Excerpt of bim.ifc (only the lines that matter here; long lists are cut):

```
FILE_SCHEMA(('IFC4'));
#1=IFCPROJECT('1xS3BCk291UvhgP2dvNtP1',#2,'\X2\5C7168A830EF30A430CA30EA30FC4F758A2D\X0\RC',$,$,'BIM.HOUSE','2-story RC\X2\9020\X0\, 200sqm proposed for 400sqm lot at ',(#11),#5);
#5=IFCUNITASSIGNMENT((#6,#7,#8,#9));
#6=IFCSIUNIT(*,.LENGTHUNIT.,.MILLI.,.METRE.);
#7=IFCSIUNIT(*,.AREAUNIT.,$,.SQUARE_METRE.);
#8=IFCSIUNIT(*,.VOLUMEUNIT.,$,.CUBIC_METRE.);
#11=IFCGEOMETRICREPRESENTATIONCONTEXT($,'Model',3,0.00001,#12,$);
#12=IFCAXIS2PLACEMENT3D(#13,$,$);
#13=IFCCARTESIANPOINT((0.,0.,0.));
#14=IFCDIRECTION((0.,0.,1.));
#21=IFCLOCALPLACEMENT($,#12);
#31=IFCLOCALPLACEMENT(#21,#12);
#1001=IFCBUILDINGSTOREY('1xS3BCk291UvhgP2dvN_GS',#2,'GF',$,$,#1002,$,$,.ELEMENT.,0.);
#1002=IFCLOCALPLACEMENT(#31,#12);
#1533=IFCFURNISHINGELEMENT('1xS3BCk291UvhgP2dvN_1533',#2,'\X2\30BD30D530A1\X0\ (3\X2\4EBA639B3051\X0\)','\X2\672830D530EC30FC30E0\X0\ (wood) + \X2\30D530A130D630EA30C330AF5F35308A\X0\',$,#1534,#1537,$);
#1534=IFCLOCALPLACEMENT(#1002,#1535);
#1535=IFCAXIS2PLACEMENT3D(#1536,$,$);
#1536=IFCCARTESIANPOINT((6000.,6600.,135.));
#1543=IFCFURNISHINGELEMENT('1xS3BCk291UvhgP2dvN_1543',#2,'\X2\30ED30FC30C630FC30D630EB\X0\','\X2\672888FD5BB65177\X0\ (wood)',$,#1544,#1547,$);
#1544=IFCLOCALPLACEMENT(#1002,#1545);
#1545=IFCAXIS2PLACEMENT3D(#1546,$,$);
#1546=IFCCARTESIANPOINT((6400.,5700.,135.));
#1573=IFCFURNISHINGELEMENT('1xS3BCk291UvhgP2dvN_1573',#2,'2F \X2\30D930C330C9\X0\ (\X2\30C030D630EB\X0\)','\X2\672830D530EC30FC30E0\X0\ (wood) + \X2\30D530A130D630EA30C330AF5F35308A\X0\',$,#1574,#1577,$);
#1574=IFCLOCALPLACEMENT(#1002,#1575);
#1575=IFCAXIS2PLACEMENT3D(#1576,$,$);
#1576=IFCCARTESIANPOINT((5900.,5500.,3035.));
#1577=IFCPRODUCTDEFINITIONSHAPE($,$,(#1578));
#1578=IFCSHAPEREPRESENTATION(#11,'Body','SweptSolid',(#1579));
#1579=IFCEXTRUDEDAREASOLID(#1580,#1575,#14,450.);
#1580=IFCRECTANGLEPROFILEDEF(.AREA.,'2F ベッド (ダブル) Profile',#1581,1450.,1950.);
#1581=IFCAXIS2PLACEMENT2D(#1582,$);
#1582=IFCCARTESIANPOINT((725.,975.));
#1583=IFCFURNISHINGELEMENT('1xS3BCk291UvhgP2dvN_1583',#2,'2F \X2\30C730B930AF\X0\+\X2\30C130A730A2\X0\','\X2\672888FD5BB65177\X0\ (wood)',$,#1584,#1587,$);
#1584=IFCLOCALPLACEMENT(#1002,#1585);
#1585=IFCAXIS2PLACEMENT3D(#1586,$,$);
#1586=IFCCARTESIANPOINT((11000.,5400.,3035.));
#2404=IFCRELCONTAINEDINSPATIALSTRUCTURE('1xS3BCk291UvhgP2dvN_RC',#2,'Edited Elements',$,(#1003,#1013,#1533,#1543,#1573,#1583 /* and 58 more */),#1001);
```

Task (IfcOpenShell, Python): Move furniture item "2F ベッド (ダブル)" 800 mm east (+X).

```python
import ifcopenshell
import ifcopenshell.api.geometry
import ifcopenshell.util.placement

model = ifcopenshell.open("bim.ifc")

item = model.by_guid("1xS3BCk291UvhgP2dvN_1573")
matrix = ifcopenshell.util.placement.get_local_placement(item.ObjectPlacement)
matrix[0, 3] += 800.0
ifcopenshell.api.geometry.edit_object_placement(model, product=item, matrix=matrix, is_si=False)

print(ifcopenshell.util.placement.get_local_placement(item.ObjectPlacement).round(3) + 0.0)

model.write("bim-out.ifc")
```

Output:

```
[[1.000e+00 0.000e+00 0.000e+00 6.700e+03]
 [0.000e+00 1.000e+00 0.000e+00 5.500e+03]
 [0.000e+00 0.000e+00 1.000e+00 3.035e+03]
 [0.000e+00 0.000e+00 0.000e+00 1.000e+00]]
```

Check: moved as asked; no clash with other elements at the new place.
